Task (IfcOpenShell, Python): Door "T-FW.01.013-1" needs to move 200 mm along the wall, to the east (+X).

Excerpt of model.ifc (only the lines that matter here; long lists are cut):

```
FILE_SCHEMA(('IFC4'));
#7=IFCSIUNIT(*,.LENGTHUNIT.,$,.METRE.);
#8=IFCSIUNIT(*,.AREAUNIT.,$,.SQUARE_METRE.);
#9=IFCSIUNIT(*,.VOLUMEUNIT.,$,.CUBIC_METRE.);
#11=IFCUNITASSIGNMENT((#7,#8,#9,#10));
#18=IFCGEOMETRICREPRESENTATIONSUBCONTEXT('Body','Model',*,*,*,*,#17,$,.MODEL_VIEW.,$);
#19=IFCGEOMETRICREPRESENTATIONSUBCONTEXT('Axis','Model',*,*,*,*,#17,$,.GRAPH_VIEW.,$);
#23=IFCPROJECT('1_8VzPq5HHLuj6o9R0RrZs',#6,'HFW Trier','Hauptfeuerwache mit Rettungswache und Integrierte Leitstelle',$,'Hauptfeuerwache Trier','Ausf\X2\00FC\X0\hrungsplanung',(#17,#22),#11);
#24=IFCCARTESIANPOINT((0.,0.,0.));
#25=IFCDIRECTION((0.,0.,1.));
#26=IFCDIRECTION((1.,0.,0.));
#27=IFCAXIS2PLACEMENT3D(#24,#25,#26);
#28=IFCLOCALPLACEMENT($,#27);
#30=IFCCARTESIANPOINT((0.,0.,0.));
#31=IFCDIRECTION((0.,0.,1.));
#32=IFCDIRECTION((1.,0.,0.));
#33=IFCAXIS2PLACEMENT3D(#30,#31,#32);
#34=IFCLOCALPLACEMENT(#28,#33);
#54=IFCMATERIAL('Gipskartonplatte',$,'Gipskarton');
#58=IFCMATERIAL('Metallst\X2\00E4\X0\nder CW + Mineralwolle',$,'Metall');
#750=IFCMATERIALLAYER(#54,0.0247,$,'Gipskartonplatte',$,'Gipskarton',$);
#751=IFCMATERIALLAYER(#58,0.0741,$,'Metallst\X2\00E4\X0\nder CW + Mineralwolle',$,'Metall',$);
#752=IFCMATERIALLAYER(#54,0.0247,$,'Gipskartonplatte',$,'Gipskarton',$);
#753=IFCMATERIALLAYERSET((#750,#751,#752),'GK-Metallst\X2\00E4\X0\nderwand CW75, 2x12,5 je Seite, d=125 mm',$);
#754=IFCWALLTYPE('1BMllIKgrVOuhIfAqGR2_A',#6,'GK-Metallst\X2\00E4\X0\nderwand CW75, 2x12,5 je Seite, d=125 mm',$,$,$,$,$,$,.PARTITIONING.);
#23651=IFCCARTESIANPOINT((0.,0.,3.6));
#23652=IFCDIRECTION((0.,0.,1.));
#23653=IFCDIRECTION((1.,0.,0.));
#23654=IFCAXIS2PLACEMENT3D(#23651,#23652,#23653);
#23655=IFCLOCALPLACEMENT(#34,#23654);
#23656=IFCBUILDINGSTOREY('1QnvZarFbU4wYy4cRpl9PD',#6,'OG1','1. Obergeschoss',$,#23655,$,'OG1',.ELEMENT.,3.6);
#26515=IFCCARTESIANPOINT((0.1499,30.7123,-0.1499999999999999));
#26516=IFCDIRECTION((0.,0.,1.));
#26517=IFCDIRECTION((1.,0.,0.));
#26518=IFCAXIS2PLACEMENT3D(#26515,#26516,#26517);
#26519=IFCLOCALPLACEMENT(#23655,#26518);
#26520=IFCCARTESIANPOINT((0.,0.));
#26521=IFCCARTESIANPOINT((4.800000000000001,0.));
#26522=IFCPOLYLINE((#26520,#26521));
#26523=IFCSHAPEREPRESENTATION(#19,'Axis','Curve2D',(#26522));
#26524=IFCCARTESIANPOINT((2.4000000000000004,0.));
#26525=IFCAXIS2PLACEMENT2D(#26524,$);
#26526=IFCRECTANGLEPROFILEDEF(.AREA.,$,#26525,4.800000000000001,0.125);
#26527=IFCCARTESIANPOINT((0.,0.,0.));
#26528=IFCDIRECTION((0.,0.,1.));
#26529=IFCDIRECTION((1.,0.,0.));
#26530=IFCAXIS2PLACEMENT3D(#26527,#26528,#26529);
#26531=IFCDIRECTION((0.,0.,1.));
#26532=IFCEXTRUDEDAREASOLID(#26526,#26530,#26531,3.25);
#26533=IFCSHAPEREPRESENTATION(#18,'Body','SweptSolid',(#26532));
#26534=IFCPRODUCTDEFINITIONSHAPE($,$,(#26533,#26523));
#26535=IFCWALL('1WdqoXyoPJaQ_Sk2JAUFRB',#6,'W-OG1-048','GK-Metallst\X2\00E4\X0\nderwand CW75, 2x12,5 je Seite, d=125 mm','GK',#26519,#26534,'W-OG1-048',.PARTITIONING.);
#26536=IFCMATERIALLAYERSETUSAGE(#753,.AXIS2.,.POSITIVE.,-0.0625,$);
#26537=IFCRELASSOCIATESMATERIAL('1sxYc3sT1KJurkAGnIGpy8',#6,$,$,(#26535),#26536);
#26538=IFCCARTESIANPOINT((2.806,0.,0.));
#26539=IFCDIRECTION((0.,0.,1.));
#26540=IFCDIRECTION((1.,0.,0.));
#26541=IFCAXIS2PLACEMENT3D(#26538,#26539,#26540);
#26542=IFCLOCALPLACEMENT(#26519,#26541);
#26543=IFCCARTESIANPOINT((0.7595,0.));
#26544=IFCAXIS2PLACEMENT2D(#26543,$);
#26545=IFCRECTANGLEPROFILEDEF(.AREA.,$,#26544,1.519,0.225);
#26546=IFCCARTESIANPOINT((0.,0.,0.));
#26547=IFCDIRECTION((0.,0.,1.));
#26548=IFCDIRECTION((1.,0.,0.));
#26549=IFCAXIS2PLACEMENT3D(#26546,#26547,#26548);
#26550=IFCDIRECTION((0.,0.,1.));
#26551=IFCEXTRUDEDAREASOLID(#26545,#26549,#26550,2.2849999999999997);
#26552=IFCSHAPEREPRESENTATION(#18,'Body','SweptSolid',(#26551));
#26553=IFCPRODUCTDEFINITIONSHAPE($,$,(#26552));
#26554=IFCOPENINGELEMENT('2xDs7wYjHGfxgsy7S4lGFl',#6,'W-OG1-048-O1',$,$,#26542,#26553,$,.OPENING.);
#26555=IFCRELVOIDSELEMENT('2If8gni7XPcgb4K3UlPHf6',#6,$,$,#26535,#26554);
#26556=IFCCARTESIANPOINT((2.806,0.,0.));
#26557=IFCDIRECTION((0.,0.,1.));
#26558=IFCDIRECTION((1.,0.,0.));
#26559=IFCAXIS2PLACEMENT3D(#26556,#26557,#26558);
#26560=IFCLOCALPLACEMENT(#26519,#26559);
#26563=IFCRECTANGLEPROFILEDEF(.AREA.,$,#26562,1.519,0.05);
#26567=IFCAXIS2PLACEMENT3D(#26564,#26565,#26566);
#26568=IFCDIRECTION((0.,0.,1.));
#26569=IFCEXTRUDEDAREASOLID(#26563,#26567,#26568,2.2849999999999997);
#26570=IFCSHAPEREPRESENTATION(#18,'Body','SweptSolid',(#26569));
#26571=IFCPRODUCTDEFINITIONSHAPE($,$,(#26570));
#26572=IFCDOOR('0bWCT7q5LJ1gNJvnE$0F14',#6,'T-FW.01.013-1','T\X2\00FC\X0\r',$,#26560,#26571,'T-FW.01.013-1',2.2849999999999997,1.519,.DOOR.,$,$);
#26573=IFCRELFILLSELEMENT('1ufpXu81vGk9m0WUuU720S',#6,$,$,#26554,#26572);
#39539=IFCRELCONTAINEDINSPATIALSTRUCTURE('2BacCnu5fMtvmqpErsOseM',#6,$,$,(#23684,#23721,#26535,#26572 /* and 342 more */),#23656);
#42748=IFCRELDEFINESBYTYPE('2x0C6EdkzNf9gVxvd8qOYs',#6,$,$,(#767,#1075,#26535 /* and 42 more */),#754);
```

```python
import ifcopenshell
import ifcopenshell.api.geometry
import ifcopenshell.util.placement
import ifcopenshell.util.unit

model = ifcopenshell.open("model.ifc")
unit_scale = ifcopenshell.util.unit.calculate_unit_scale(model)

door = model.by_id(26572)
opening = door.FillsVoids[0].RelatingOpeningElement
wall = opening.VoidsElements[0].RelatingBuildingElement

wall_matrix = ifcopenshell.util.placement.get_local_placement(wall.ObjectPlacement)
shift = wall_matrix[:3, 0] * 0.2 / unit_scale
before = ifcopenshell.util.placement.get_local_placement(door.ObjectPlacement)[:3, 3].copy()

# The door is not placed relative to its opening, so move both.
for product in (opening, door):
    matrix = ifcopenshell.util.placement.get_local_placement(product.ObjectPlacement)
    matrix[:3, 3] += shift
    ifcopenshell.api.geometry.edit_object_placement(model, product=product, matrix=matrix, is_si=False)

after = ifcopenshell.util.placement.get_local_placement(door.ObjectPlacement)[:3, 3]
print("door moved by", (after - before).round(3) + 0.0)

model.write("model_v2.ifc")
```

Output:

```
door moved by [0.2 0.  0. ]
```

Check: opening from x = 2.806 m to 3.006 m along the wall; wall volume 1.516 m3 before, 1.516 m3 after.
